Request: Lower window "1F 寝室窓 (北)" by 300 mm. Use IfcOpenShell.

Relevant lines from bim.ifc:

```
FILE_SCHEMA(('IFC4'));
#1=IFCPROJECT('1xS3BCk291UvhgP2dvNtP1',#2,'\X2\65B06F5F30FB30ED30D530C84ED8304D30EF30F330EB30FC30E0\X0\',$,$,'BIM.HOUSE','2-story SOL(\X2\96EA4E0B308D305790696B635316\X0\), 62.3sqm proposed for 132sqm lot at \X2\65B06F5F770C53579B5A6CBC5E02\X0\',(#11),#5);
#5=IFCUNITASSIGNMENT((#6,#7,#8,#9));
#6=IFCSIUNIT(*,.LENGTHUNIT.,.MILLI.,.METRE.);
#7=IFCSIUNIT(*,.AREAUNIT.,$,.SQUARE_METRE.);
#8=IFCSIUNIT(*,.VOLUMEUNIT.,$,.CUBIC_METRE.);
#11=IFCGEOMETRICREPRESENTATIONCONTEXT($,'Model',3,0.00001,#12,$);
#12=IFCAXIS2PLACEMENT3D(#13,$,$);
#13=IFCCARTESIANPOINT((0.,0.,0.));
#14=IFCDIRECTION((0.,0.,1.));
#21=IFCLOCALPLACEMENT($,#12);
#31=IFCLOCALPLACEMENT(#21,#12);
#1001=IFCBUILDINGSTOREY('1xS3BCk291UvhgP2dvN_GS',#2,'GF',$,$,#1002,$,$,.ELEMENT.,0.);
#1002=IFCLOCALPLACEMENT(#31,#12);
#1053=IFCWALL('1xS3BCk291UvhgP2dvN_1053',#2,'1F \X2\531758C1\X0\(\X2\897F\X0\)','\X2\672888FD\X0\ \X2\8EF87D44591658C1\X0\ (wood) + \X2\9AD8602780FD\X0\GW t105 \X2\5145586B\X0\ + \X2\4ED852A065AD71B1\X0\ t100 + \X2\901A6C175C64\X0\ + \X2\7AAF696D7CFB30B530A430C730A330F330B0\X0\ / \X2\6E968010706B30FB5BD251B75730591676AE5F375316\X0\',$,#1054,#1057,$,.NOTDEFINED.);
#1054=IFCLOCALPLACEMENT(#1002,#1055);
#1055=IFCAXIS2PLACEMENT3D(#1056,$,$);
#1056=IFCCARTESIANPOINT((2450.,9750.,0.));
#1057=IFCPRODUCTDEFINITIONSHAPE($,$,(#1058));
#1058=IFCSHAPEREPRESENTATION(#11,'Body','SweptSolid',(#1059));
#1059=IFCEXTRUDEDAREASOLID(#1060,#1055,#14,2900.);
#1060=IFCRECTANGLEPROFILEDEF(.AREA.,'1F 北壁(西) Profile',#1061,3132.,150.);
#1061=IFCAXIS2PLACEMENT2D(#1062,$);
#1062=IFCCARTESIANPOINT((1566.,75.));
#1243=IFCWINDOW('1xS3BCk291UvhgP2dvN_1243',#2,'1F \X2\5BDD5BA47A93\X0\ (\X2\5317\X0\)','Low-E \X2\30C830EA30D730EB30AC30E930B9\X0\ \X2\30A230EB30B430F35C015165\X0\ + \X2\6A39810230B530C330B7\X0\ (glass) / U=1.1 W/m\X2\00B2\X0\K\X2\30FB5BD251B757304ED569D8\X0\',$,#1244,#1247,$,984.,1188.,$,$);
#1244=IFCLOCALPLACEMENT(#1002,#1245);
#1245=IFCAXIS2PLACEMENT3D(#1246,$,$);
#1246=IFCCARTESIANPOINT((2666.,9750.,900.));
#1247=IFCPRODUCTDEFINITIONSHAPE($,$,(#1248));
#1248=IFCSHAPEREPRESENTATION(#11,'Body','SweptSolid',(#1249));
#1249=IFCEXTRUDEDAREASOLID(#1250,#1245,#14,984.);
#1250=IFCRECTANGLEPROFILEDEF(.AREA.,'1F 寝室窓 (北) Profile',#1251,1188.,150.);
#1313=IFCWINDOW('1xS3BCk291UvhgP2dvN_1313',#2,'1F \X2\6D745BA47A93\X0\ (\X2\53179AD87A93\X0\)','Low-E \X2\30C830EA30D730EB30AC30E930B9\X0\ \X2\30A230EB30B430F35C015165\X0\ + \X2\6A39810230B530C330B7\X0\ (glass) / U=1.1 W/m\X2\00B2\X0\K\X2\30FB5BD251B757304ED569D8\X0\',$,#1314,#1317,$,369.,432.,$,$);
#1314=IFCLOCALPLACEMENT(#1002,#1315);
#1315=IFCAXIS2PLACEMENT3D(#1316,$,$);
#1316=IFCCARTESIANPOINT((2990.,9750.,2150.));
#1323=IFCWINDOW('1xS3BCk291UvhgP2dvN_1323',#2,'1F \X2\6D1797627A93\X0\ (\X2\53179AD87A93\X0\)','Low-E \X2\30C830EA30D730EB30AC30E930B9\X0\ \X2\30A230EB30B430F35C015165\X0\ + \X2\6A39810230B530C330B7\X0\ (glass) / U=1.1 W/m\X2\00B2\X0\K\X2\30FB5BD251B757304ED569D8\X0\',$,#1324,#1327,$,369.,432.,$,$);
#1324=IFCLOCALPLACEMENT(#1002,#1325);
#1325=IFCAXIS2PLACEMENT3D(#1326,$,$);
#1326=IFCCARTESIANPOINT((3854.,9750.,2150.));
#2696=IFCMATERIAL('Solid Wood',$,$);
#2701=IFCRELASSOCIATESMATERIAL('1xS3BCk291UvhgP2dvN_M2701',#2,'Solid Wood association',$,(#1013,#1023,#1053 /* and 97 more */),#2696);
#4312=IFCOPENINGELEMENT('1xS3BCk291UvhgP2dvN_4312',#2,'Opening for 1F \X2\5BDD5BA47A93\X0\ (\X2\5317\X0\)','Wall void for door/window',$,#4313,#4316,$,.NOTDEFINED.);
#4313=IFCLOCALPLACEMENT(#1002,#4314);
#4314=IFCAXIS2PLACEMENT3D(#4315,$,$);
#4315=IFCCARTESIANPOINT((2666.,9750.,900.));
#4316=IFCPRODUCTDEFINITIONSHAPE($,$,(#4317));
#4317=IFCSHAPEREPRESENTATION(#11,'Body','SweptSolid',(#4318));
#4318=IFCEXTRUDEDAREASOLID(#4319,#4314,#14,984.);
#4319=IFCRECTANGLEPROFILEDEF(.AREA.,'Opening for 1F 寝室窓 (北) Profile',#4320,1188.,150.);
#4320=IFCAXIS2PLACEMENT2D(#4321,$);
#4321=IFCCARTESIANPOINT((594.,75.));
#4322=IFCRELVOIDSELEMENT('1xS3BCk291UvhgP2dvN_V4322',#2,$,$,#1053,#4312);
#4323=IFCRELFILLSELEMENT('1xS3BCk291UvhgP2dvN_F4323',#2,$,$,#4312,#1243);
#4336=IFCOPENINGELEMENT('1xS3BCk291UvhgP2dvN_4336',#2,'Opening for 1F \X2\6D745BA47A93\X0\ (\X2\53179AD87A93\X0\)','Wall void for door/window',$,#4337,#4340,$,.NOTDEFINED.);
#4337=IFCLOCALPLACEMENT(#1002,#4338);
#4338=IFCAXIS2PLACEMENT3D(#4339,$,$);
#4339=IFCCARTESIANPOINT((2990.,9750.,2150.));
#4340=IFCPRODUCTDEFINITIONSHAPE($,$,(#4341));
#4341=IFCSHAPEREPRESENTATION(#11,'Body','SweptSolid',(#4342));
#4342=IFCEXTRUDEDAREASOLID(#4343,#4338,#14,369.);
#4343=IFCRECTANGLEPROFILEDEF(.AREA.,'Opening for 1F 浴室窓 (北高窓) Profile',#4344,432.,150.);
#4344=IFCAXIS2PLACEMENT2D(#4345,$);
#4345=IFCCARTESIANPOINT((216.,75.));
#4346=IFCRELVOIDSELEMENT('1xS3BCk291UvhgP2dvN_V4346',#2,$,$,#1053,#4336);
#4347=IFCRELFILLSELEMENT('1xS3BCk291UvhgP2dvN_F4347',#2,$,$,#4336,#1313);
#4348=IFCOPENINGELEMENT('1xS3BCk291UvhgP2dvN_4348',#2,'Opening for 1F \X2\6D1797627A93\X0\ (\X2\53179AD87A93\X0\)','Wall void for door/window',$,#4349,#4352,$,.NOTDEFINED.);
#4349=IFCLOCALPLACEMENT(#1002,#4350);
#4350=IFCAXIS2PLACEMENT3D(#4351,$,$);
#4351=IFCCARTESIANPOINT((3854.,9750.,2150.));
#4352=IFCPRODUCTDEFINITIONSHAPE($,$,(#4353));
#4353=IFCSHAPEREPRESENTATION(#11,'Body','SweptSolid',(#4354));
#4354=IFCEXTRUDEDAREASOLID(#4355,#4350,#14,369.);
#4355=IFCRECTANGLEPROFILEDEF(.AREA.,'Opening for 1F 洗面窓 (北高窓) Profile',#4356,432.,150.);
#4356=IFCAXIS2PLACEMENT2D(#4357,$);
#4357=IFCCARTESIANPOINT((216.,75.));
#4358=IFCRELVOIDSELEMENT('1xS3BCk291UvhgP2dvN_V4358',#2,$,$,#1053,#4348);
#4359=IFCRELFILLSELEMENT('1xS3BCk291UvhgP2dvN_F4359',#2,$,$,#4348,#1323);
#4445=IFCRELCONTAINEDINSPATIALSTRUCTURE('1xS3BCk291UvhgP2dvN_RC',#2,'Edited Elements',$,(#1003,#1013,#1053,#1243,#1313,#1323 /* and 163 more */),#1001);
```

```python
import numpy as np
import ifcopenshell
import ifcopenshell.api.geometry
import ifcopenshell.util.placement
import ifcopenshell.util.unit

model = ifcopenshell.open("bim.ifc")
unit_scale = ifcopenshell.util.unit.calculate_unit_scale(model)

window = model.by_guid("1xS3BCk291UvhgP2dvN_1243")
opening = window.FillsVoids[0].RelatingOpeningElement
dz = -300.0

shift = np.array([0.0, 0.0, dz])
# The window is not placed relative to its opening, so move both.
for product in (opening, window):
    matrix = ifcopenshell.util.placement.get_local_placement(product.ObjectPlacement)
    matrix[:3, 3] += shift
    ifcopenshell.api.geometry.edit_object_placement(model, product=product, matrix=matrix, is_si=False)

print(f"moved by {dz * unit_scale:+.3f} m")

model.write("bim_updated.ifc")
```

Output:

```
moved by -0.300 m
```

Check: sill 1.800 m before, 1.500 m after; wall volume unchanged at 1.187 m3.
